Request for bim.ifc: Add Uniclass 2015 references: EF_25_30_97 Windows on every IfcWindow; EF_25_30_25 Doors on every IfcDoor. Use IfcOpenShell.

First a look at what the model holds.

```python
import ifcopenshell

model = ifcopenshell.open("bim.ifc")
print(model.schema)
print("classifications:", [c.Name for c in model.by_type("IfcClassification")])
for ifc_class in ("IfcDoor", "IfcRoof", "IfcStair", "IfcWall", "IfcWindow"):
    print(ifc_class, len(model.by_type(ifc_class)))
```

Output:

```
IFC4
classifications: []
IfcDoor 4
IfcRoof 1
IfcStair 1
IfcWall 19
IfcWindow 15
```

```python
import ifcopenshell
import ifcopenshell.api.classification

model = ifcopenshell.open("bim.ifc")

system = ifcopenshell.api.classification.add_classification(model, classification="Uniclass 2015")

codes = {
    "IfcWindow": ("EF_25_30_97", "Windows"),
    "IfcDoor": ("EF_25_30_25", "Doors"),
}
for ifc_class, (code, name) in codes.items():
    products = model.by_type(ifc_class)
    ifcopenshell.api.classification.add_reference(
        model, products=products, classification=system, identification=code, name=name
    )
    print(code, len(products))

model.write("bim_updated.ifc")
```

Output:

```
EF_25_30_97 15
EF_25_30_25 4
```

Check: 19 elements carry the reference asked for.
